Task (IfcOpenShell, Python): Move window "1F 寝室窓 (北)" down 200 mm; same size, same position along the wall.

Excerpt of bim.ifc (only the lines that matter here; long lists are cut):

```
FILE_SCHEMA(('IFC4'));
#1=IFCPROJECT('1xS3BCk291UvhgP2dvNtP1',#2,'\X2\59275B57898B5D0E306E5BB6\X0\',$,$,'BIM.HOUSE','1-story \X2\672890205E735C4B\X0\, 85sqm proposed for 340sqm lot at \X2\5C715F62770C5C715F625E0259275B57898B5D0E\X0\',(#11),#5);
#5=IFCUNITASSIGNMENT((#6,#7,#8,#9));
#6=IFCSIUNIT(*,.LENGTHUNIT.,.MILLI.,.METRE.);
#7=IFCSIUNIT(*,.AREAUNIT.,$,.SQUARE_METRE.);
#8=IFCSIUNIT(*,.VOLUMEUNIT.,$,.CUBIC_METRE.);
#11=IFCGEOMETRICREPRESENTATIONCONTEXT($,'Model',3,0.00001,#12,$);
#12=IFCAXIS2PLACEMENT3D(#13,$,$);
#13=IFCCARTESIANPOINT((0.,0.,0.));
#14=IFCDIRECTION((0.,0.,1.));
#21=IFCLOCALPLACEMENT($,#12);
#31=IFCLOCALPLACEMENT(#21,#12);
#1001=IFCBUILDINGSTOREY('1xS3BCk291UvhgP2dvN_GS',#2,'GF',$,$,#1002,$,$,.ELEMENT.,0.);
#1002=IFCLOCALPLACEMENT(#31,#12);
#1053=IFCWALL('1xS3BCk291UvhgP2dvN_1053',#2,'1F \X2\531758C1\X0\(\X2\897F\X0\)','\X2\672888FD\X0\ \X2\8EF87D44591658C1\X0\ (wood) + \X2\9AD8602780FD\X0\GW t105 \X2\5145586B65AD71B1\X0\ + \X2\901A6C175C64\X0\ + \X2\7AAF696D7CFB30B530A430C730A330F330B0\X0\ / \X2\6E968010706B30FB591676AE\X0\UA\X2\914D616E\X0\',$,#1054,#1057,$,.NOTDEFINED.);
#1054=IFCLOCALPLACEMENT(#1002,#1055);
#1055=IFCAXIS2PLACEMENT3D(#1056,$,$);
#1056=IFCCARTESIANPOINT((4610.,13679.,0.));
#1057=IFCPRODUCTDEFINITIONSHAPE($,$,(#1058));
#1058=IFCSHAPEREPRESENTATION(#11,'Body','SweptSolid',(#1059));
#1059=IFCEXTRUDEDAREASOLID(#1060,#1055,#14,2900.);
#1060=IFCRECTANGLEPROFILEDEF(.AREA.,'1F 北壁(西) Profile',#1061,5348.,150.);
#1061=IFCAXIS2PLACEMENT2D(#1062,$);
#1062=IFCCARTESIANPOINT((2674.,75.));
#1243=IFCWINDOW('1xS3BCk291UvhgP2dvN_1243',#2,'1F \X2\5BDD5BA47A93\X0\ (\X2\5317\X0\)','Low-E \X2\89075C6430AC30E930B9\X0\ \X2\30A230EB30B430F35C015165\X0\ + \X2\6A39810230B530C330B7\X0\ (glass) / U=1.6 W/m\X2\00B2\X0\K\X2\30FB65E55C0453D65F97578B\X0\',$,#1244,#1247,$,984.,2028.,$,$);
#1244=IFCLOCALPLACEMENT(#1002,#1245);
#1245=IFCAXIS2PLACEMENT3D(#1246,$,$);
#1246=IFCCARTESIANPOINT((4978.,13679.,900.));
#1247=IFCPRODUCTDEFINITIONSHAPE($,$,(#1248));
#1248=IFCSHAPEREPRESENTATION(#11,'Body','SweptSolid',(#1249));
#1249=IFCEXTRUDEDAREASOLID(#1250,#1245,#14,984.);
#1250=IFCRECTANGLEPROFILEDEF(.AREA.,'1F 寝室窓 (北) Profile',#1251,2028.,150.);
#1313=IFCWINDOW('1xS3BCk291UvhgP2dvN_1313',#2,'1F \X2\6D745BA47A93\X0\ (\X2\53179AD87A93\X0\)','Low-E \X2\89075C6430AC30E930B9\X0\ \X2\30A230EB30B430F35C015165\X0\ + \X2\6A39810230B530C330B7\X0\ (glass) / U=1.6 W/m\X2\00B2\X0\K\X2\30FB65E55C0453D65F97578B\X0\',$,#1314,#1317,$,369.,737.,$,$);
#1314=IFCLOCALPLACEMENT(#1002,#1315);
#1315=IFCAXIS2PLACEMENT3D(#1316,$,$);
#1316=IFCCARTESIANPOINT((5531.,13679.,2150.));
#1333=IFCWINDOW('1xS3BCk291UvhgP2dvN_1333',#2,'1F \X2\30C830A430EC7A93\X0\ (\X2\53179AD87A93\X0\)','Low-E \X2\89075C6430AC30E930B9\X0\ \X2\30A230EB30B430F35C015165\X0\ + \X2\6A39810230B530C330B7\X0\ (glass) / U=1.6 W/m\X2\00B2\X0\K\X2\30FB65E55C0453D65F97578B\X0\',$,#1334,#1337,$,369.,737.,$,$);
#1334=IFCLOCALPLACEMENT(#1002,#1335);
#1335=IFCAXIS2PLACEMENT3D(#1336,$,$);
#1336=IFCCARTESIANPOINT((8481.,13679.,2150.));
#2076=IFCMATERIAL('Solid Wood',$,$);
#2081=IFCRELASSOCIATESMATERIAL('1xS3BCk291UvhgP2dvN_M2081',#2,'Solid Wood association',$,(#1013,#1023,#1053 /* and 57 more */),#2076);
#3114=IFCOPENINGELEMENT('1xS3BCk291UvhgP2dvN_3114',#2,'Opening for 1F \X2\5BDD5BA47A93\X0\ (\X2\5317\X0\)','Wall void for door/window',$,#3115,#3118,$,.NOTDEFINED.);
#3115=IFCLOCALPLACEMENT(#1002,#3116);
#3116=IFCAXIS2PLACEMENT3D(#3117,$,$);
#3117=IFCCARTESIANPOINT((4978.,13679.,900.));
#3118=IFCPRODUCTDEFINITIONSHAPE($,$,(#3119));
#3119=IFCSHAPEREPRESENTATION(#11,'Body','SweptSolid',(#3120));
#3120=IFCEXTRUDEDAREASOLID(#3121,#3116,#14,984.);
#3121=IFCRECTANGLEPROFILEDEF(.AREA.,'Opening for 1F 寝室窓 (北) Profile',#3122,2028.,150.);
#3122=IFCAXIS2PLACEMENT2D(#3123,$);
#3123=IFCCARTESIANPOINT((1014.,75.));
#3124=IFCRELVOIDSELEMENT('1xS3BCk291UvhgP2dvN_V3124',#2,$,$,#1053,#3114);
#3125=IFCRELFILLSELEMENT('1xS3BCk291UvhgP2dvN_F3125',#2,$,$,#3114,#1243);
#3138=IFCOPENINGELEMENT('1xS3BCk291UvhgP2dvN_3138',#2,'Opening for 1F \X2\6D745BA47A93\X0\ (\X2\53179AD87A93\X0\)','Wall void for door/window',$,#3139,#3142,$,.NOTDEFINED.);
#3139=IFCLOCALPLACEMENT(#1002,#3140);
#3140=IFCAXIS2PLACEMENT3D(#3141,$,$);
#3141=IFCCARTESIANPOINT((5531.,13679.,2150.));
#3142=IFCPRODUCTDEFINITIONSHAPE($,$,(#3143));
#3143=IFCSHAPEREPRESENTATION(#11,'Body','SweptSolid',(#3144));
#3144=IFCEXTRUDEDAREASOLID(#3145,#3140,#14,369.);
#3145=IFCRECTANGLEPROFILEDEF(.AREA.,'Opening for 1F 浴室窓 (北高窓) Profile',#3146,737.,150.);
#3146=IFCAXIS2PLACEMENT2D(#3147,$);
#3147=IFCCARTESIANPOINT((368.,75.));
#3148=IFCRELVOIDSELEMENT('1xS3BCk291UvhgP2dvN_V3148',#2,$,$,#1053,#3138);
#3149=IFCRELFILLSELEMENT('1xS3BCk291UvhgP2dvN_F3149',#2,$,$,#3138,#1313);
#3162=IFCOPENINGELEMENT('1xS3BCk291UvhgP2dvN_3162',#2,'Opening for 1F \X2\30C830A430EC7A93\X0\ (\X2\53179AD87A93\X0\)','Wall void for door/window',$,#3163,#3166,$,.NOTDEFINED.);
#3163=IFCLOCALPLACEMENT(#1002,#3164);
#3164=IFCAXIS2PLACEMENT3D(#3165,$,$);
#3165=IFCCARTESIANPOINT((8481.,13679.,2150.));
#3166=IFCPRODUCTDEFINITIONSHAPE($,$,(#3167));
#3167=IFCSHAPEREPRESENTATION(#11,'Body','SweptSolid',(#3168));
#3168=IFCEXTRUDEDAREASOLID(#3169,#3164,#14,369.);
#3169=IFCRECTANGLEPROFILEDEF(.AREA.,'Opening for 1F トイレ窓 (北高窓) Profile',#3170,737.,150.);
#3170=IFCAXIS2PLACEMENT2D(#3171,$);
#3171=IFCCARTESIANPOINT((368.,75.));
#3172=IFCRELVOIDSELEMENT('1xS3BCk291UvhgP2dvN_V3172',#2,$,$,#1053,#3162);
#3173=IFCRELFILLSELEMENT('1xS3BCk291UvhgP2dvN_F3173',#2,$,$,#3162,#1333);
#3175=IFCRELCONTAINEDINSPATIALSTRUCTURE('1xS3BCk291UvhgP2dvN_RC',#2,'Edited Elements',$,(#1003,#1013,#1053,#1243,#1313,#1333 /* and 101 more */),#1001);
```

```python
import numpy as np
import ifcopenshell
import ifcopenshell.api.geometry
import ifcopenshell.util.placement
import ifcopenshell.util.unit

model = ifcopenshell.open("bim.ifc")
unit_scale = ifcopenshell.util.unit.calculate_unit_scale(model)

window = model.by_guid("1xS3BCk291UvhgP2dvN_1243")
opening = window.FillsVoids[0].RelatingOpeningElement
dz = -0.2 / unit_scale

shift = np.array([0.0, 0.0, dz])
# The window is not placed relative to its opening, so move both.
for product in (opening, window):
    matrix = ifcopenshell.util.placement.get_local_placement(product.ObjectPlacement)
    matrix[:3, 3] += shift
    ifcopenshell.api.geometry.edit_object_placement(model, product=product, matrix=matrix, is_si=False)

print(f"moved by {dz * unit_scale:+.3f} m")

model.write("bim_updated.ifc")
```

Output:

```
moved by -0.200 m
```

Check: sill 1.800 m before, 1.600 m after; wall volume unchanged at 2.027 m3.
